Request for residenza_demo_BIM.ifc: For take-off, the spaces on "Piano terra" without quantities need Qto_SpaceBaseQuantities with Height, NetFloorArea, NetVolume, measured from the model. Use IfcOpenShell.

First a look at what the model holds.

```python
import ifcopenshell
import ifcopenshell.util.element
import ifcopenshell.util.unit

model = ifcopenshell.open("residenza_demo_BIM.ifc")
print(model.schema)
for unit_type in ("LENGTHUNIT", "AREAUNIT", "VOLUMEUNIT"):
    print(unit_type, ifcopenshell.util.unit.calculate_unit_scale(model, unit_type))
storey = next(s for s in model.by_type("IfcBuildingStorey") if s.Name == "Piano terra")
spaces = [e for e in ifcopenshell.util.element.get_decomposition(storey) if e.is_a("IfcSpace")]
for e in sorted(spaces, key=lambda e: e.id()):
    print(e.id(), e.is_a(), e.Name, list(ifcopenshell.util.element.get_psets(e, qtos_only=True)), sep=" | ")
```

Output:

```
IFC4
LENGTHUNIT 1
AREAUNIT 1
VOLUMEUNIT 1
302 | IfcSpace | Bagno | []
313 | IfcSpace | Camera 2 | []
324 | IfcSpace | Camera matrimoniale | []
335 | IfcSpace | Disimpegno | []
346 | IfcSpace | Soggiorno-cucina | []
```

```python
import ifcopenshell
import ifcopenshell.api.pset
import ifcopenshell.geom
import ifcopenshell.util.element
import ifcopenshell.util.shape
import ifcopenshell.util.unit

model = ifcopenshell.open("residenza_demo_BIM.ifc")
unit_scale = ifcopenshell.util.unit.calculate_unit_scale(model)
area_scale = ifcopenshell.util.unit.calculate_unit_scale(model, "AREAUNIT")
volume_scale = ifcopenshell.util.unit.calculate_unit_scale(model, "VOLUMEUNIT")
settings = ifcopenshell.geom.settings()

storey = next(s for s in model.by_type("IfcBuildingStorey") if s.Name == "Piano terra")
spaces = [e for e in ifcopenshell.util.element.get_decomposition(storey) if e.is_a("IfcSpace")]

for e in sorted(spaces, key=lambda e: e.id()):
    if ifcopenshell.util.element.get_psets(e, qtos_only=True, should_inherit=False):
        continue
    # Geometry comes back in metres, in the element's own axes.
    shape = ifcopenshell.geom.create_shape(settings, e)
    values = {
        "Height": ifcopenshell.util.shape.get_z(shape.geometry) / unit_scale,
        "NetFloorArea": ifcopenshell.util.shape.get_footprint_area(shape.geometry) / area_scale,
        "NetVolume": ifcopenshell.util.shape.get_volume(shape.geometry) / volume_scale,
    }
    qto = ifcopenshell.api.pset.add_qto(model, product=e, name="Qto_SpaceBaseQuantities")
    ifcopenshell.api.pset.edit_qto(model, qto=qto, properties=values)
    print(e.id(), {k: round(v, 3) for k, v in values.items()})

model.write("residenza_demo_BIM-out.ifc")
```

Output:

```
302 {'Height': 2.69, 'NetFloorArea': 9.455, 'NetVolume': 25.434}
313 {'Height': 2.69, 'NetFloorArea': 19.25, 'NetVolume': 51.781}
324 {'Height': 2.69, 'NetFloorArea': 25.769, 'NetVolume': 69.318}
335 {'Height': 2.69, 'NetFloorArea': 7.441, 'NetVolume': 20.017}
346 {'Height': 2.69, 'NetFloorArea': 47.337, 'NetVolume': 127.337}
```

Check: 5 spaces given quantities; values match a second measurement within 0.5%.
